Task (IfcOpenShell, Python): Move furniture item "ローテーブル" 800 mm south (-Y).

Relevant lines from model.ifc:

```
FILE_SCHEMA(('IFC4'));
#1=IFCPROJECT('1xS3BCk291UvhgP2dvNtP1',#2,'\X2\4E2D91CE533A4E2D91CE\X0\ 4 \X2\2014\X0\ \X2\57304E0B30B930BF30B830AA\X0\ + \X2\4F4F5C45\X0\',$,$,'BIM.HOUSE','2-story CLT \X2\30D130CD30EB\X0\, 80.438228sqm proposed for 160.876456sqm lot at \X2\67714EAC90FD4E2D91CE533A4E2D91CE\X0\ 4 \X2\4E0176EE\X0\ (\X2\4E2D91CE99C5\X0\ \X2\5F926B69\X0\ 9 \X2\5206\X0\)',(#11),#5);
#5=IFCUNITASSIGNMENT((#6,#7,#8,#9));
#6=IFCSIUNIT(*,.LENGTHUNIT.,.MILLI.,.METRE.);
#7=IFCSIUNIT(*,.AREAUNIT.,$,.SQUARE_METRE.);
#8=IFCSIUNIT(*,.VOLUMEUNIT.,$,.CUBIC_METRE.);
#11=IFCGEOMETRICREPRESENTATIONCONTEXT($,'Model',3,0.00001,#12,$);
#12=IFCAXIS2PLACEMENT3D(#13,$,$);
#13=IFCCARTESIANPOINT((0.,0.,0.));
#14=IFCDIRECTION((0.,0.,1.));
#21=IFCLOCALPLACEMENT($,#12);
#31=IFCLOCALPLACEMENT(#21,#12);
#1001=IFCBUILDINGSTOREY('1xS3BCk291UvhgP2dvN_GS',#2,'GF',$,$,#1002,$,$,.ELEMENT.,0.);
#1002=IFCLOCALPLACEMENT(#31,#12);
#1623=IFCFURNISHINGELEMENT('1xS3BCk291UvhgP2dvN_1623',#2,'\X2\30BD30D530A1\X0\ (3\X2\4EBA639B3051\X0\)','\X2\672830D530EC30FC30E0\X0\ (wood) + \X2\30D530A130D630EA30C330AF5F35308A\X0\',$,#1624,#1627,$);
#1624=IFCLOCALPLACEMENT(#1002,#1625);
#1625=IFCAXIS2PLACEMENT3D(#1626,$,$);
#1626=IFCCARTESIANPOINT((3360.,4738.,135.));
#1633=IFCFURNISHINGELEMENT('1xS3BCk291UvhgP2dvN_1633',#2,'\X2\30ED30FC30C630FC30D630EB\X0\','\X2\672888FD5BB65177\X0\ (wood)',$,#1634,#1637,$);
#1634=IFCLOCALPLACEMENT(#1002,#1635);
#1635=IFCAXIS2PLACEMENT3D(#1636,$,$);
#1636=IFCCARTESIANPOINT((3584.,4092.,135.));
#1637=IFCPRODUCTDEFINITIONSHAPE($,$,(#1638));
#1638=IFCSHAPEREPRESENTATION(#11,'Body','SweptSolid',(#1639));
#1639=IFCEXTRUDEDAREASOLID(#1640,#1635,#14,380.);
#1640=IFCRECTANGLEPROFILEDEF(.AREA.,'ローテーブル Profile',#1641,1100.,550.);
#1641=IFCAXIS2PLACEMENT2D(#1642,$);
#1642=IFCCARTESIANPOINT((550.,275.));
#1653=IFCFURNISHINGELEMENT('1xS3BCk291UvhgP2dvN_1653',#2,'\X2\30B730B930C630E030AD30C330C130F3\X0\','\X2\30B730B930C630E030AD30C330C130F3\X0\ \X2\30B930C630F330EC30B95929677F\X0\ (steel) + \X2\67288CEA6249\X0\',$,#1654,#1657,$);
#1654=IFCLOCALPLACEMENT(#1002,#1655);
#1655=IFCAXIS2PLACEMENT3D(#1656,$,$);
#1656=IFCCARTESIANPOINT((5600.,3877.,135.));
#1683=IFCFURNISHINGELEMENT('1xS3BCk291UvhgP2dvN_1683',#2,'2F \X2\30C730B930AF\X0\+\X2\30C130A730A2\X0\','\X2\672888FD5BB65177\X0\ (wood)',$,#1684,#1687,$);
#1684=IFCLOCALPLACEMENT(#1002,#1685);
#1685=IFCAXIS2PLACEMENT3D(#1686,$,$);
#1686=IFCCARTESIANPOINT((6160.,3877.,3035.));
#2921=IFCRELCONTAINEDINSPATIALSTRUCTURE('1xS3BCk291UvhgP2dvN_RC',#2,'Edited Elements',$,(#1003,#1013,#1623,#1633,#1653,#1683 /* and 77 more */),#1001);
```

```python
import ifcopenshell
import ifcopenshell.api.geometry
import ifcopenshell.util.placement

model = ifcopenshell.open("model.ifc")

item = model.by_guid("1xS3BCk291UvhgP2dvN_1633")
matrix = ifcopenshell.util.placement.get_local_placement(item.ObjectPlacement)
matrix[1, 3] -= 800.0
ifcopenshell.api.geometry.edit_object_placement(model, product=item, matrix=matrix, is_si=False)

print(ifcopenshell.util.placement.get_local_placement(item.ObjectPlacement).round(3) + 0.0)

model.write("model_updated.ifc")
```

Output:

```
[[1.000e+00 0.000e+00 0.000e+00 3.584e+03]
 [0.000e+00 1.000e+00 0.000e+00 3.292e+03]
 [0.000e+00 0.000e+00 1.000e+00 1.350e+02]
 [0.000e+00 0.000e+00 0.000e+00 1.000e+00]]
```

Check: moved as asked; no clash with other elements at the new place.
